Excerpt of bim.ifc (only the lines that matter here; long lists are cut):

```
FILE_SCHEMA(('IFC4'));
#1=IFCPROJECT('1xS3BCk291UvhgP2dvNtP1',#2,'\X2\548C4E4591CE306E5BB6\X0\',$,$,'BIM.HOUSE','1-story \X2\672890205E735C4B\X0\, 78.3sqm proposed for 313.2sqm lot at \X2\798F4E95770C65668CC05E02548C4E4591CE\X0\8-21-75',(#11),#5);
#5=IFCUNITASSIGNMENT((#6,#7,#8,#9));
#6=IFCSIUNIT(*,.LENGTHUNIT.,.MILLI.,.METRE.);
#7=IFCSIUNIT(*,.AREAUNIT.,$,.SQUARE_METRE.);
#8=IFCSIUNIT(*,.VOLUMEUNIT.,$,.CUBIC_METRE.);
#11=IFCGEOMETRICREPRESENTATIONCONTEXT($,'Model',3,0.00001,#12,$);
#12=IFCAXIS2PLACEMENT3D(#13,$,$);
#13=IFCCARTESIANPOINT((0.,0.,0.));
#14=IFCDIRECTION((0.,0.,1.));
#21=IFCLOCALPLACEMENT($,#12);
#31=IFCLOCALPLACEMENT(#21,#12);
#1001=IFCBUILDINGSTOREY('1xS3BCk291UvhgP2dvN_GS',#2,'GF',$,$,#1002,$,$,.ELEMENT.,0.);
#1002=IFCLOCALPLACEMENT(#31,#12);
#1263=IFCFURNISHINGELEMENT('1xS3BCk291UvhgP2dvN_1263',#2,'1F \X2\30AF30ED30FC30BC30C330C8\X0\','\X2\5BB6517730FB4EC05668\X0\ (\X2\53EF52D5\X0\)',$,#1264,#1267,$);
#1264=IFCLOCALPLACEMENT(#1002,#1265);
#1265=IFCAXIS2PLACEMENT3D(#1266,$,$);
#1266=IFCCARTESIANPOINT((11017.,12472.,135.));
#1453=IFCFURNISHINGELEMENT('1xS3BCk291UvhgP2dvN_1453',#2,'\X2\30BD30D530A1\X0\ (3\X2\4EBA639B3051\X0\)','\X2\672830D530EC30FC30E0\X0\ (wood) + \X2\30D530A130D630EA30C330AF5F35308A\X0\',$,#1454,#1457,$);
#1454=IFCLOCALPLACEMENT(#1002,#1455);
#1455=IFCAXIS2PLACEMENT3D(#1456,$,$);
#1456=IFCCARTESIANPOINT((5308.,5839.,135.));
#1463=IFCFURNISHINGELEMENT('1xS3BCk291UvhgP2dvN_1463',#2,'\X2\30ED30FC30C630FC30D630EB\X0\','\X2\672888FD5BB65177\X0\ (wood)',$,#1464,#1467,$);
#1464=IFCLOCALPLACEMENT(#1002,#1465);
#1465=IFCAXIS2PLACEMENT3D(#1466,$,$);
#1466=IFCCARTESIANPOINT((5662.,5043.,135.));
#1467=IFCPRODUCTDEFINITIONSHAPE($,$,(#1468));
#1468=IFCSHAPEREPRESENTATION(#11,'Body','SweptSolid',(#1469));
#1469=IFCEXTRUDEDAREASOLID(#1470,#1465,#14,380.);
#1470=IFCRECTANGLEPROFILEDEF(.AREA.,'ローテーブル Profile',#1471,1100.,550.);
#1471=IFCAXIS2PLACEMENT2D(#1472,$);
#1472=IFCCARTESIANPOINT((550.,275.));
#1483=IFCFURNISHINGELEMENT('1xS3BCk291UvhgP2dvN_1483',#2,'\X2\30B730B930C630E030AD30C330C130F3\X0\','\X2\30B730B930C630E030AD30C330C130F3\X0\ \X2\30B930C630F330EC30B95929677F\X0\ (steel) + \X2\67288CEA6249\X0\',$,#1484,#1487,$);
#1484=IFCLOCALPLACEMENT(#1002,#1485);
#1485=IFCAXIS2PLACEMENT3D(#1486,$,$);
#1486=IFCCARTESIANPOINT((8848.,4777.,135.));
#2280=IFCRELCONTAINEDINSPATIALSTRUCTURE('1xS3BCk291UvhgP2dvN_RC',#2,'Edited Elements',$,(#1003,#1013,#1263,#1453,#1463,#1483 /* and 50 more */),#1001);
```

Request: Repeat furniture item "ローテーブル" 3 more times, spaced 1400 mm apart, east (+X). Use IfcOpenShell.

```python
import numpy as np
import ifcopenshell
import ifcopenshell.api.geometry
import ifcopenshell.api.root
import ifcopenshell.util.element
import ifcopenshell.util.placement

model = ifcopenshell.open("bim.ifc")


def reuse_history(source, copy):
    """copy_class also copies each property set's owner history, people and application; keep the originals."""
    for rel in copy.IsDefinedBy:
        if rel.is_a("IfcRelDefinesByProperties") and (history := rel.RelatingPropertyDefinition.OwnerHistory):
            rel.RelatingPropertyDefinition.OwnerHistory = source.OwnerHistory
            ifcopenshell.util.element.remove_deep2(model, history)


source = model.by_guid("1xS3BCk291UvhgP2dvN_1463")
base = ifcopenshell.util.placement.get_local_placement(source.ObjectPlacement)
step = np.array([1.0, 0.0, 0.0]) * 1400.0

for i in range(1, 4):
    copy = ifcopenshell.api.root.copy_class(model, product=source)
    copy.Representation = ifcopenshell.util.element.copy_deep(
        model, source.Representation, exclude=["IfcGeometricRepresentationContext", "IfcRepresentationMap"]
    )
    reuse_history(source, copy)
    matrix = base.copy()
    matrix[:3, 3] += i * step
    print("added at", matrix[:3, 3].round(3) + 0.0)
    ifcopenshell.api.geometry.edit_object_placement(model, product=copy, matrix=matrix, is_si=False)

model.write("bim_v2.ifc")
```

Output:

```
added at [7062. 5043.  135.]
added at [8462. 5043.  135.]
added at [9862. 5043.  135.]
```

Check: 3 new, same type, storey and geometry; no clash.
